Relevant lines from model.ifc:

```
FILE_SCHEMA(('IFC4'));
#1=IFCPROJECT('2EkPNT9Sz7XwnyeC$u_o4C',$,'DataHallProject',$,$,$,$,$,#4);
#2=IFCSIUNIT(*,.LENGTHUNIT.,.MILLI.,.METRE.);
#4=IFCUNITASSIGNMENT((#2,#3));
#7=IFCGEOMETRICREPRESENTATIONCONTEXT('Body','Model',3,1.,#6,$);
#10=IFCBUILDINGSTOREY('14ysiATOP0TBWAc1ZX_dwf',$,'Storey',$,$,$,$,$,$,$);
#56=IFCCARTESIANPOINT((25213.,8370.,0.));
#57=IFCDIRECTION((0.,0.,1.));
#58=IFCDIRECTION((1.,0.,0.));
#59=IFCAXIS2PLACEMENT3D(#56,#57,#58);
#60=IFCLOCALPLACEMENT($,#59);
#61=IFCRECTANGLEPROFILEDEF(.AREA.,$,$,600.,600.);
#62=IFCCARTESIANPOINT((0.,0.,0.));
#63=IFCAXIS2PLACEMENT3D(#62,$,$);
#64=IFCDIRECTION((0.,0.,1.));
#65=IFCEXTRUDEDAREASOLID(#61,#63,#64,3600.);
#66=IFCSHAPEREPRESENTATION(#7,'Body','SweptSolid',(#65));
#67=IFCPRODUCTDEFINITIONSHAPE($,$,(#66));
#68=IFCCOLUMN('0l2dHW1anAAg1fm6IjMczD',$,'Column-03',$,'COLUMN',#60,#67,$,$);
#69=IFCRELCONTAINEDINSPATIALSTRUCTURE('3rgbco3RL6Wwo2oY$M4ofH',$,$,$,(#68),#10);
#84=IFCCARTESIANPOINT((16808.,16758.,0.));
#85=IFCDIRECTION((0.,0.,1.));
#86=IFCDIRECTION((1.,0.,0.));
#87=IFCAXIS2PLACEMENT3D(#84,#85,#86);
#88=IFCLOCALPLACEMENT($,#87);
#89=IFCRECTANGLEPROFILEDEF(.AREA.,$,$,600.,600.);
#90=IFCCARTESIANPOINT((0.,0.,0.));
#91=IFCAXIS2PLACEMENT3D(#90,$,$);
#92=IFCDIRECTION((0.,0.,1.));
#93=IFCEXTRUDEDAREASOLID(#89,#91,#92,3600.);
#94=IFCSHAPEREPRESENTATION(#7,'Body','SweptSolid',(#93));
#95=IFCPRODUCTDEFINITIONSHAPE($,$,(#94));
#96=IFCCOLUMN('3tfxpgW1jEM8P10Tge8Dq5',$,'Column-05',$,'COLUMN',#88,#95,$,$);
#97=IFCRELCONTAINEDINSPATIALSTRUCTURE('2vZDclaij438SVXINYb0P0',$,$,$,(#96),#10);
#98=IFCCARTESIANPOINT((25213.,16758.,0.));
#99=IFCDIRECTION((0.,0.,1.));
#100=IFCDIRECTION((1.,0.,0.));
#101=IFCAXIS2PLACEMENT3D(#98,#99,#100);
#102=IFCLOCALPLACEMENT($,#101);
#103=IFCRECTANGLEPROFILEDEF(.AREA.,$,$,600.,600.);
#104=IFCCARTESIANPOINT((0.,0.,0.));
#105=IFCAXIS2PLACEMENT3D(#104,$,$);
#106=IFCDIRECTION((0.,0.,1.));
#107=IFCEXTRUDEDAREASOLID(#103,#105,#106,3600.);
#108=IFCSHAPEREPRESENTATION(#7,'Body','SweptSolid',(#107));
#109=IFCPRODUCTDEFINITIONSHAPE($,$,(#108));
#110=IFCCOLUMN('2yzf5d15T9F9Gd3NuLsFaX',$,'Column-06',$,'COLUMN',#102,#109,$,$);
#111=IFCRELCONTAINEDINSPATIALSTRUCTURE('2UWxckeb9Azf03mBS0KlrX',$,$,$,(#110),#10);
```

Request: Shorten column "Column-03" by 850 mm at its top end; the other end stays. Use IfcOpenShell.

```python
import ifcopenshell
import ifcopenshell.util.unit

model = ifcopenshell.open("model.ifc")
unit_scale = ifcopenshell.util.unit.calculate_unit_scale(model)

member = model.by_guid("0l2dHW1anAAg1fm6IjMczD")
change = -0.85 / unit_scale

# The extrusion runs towards the end named, so only its depth changes.
body = next(r for r in member.Representation.Representations if r.RepresentationIdentifier == "Body")
solid = body.Items[0]
old_length = solid.Depth
solid.Depth += change

print(f"length {old_length:g} -> {solid.Depth:g}")

model.write("model-out.ifc")
```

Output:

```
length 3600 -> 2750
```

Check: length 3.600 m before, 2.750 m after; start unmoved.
